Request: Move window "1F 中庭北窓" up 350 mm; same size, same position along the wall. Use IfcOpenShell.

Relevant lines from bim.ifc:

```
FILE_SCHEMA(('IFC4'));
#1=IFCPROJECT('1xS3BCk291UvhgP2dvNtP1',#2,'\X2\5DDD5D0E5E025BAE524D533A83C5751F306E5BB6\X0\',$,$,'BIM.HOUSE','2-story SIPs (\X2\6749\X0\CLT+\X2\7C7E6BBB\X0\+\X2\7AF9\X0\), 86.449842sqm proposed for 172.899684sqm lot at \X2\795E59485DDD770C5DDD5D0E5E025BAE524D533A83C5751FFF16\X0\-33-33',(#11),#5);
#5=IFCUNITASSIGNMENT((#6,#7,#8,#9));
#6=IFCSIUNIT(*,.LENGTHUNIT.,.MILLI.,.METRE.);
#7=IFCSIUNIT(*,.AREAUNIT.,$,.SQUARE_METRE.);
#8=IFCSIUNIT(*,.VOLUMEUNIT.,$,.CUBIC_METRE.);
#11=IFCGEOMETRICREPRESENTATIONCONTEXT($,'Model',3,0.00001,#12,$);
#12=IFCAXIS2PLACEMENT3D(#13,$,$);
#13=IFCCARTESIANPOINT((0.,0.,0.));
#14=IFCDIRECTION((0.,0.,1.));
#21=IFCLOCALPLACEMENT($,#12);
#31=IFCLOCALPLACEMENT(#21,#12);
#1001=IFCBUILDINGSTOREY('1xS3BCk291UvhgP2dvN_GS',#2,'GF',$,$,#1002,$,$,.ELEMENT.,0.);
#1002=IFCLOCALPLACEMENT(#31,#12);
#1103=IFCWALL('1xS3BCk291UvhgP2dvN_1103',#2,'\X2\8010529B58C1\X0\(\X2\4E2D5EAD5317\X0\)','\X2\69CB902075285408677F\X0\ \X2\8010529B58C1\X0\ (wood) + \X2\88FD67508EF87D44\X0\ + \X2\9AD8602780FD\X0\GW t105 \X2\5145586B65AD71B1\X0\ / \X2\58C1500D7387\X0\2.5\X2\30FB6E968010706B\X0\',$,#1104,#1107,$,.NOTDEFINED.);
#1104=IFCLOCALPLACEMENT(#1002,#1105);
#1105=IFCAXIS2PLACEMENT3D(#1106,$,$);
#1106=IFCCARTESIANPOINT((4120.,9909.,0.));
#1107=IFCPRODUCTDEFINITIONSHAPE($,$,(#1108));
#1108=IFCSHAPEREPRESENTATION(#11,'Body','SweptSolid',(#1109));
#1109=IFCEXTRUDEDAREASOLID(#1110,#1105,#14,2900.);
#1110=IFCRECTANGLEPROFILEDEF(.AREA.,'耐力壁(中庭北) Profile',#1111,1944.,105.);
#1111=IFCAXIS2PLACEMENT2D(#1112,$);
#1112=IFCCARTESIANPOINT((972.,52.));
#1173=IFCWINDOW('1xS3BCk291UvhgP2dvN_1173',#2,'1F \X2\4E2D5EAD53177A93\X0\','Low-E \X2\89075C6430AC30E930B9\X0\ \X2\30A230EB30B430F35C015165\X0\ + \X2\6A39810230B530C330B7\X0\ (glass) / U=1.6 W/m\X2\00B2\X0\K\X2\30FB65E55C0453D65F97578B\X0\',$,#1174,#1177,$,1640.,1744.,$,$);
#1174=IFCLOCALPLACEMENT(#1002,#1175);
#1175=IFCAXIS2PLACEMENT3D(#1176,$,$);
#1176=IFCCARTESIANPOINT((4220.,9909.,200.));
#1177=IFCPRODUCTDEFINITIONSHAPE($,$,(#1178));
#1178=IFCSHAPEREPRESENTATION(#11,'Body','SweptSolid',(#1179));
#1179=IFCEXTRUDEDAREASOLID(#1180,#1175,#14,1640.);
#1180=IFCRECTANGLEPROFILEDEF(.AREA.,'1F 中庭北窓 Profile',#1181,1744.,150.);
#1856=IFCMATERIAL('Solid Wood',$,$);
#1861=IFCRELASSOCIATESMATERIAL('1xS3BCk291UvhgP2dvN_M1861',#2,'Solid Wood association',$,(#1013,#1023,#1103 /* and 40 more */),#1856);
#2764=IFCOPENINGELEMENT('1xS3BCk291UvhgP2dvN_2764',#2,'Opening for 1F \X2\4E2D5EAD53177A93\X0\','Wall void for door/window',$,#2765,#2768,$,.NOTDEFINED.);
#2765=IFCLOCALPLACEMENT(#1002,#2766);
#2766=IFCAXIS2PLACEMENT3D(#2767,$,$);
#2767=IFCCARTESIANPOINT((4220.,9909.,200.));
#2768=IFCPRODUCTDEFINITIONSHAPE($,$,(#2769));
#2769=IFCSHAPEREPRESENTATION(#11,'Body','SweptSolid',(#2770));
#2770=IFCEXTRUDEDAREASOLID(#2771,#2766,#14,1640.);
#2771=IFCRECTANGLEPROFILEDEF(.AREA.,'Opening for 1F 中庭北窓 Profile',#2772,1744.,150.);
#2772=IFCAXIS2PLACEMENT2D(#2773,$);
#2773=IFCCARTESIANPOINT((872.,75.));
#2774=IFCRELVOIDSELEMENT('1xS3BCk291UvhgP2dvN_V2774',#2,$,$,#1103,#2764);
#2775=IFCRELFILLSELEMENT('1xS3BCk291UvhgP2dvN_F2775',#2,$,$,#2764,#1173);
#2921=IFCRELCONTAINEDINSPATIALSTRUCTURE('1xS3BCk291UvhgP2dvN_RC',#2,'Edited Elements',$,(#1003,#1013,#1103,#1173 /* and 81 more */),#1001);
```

```python
import numpy as np
import ifcopenshell
import ifcopenshell.api.geometry
import ifcopenshell.util.placement
import ifcopenshell.util.unit

model = ifcopenshell.open("bim.ifc")
unit_scale = ifcopenshell.util.unit.calculate_unit_scale(model)

window = model.by_guid("1xS3BCk291UvhgP2dvN_1173")
opening = window.FillsVoids[0].RelatingOpeningElement
dz = 350.0

shift = np.array([0.0, 0.0, dz])
# The window is not placed relative to its opening, so move both.
for product in (opening, window):
    matrix = ifcopenshell.util.placement.get_local_placement(product.ObjectPlacement)
    matrix[:3, 3] += shift
    ifcopenshell.api.geometry.edit_object_placement(model, product=product, matrix=matrix, is_si=False)

print(f"moved by {dz * unit_scale:+.3f} m")

model.write("bim_edited.ifc")
```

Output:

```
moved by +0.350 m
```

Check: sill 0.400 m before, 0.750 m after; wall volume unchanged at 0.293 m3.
